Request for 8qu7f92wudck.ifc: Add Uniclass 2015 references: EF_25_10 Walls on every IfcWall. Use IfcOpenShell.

First a look at what the model holds.

```python
import ifcopenshell

model = ifcopenshell.open("8qu7f92wudck.ifc")
print(model.schema)
print("classifications:", [c.Name for c in model.by_type("IfcClassification")])
for ifc_class in ("IfcDoor", "IfcRoof", "IfcStair", "IfcWall", "IfcWindow"):
    print(ifc_class, len(model.by_type(ifc_class)))
```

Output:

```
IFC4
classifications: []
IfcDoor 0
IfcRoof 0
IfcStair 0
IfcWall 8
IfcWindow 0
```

```python
import ifcopenshell
import ifcopenshell.api.classification

model = ifcopenshell.open("8qu7f92wudck.ifc")

system = ifcopenshell.api.classification.add_classification(model, classification="Uniclass 2015")

codes = {
    "IfcWall": ("EF_25_10", "Walls"),
}
for ifc_class, (code, name) in codes.items():
    products = model.by_type(ifc_class)
    ifcopenshell.api.classification.add_reference(
        model, products=products, classification=system, identification=code, name=name
    )
    print(code, len(products))

model.write("8qu7f92wudck-out.ifc")
```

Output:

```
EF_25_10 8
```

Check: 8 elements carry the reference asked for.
